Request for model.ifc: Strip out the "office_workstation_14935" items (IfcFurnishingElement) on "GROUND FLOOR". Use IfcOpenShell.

First a look at what the model holds.

```python
import ifcopenshell
import ifcopenshell.util.element

model = ifcopenshell.open("model.ifc")
print(model.schema)
storey = next(s for s in model.by_type("IfcBuildingStorey") if s.Name == "GROUND FLOOR")
furniture = [e for e in ifcopenshell.util.element.get_decomposition(storey) if e.is_a("IfcFurnishingElement")]
seen = {}
for e in furniture:
    element_type = ifcopenshell.util.element.get_type(e)
    name = element_type.Name if element_type not in (None, e) else None
    seen[name] = seen.get(name, 0) + 1
for name, count in sorted(seen.items(), key=str):
    print(count, "x", name)
```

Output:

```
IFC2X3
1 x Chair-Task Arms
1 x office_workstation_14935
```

```python
import ifcopenshell
import ifcopenshell.api.root
import ifcopenshell.util.element

model = ifcopenshell.open("model.ifc")

storey = next(s for s in model.by_type("IfcBuildingStorey") if s.Name == "GROUND FLOOR")
furniture = [e for e in ifcopenshell.util.element.get_decomposition(storey) if e.is_a("IfcFurnishingElement")]
targets = [e for e in furniture if (t := ifcopenshell.util.element.get_type(e)) not in (None, e) and t.Name == "office_workstation_14935"]

for e in targets:
    ifcopenshell.api.root.remove_product(model, product=e)
print(len(targets), "removed")

model.write("model_updated.ifc")
```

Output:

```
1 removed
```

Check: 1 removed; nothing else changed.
